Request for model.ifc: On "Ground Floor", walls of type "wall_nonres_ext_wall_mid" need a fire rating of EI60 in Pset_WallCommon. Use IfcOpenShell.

First a look at what the model holds.

```python
import ifcopenshell
import ifcopenshell.util.element

model = ifcopenshell.open("model.ifc")
print(model.schema)
storey = next(s for s in model.by_type("IfcBuildingStorey") if s.Name == "Ground Floor")
walls = [e for e in ifcopenshell.util.element.get_decomposition(storey) if e.is_a("IfcWall")]
seen = {}
for e in walls:
    element_type = ifcopenshell.util.element.get_type(e)
    key = (element_type.Name if element_type != e and element_type else None, ifcopenshell.util.element.get_pset(e, "Pset_WallCommon", "FireRating"))
    seen[key] = seen.get(key, 0) + 1
for (name, value), count in sorted(seen.items(), key=str):
    print(count, "x", name, "|", value)
```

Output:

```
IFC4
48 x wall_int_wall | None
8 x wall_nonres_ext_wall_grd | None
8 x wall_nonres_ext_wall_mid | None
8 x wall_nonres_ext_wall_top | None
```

```python
import ifcopenshell
import ifcopenshell.api.pset
import ifcopenshell.util.element

model = ifcopenshell.open("model.ifc")

storey = next(s for s in model.by_type("IfcBuildingStorey") if s.Name == "Ground Floor")
walls = [e for e in ifcopenshell.util.element.get_decomposition(storey) if e.is_a("IfcWall")]

count = 0
for e in walls:
    element_type = ifcopenshell.util.element.get_type(e)
    if element_type in (None, e) or element_type.Name != "wall_nonres_ext_wall_mid":
        continue
    # add_pset returns the element's existing set when there is one.
    pset = ifcopenshell.api.pset.add_pset(model, product=e, name="Pset_WallCommon")
    ifcopenshell.api.pset.edit_pset(model, pset=pset, properties={"FireRating": "EI60"})
    count += 1

print(count, "walls updated")

model.write("model-out.ifc")
```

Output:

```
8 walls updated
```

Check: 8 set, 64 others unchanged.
